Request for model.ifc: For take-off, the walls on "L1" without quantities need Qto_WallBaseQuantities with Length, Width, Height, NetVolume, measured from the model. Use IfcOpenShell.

First a look at what the model holds.

```python
import ifcopenshell
import ifcopenshell.util.element
import ifcopenshell.util.unit

model = ifcopenshell.open("model.ifc")
print(model.schema)
for unit_type in ("LENGTHUNIT", "AREAUNIT", "VOLUMEUNIT"):
    print(unit_type, ifcopenshell.util.unit.calculate_unit_scale(model, unit_type))
storey = next(s for s in model.by_type("IfcBuildingStorey") if s.Name == "L1")
walls = [e for e in ifcopenshell.util.element.get_decomposition(storey) if e.is_a("IfcWall")]
for e in sorted(walls, key=lambda e: e.id()):
    print(e.id(), e.is_a(), e.Name, list(ifcopenshell.util.element.get_psets(e, qtos_only=True)), sep=" | ")
```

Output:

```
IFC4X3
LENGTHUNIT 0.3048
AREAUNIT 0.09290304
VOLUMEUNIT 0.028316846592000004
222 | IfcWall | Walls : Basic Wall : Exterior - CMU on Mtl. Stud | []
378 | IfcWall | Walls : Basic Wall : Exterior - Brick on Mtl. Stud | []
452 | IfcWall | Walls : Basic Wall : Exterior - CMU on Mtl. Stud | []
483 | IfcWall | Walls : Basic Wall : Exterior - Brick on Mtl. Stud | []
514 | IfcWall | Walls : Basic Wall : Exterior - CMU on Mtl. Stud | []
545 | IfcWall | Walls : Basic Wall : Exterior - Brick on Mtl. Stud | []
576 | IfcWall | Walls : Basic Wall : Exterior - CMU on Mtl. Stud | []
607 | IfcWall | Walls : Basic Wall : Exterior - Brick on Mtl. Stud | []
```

```python
import ifcopenshell
import ifcopenshell.api.pset
import ifcopenshell.geom
import ifcopenshell.util.element
import ifcopenshell.util.shape
import ifcopenshell.util.unit

model = ifcopenshell.open("model.ifc")
unit_scale = ifcopenshell.util.unit.calculate_unit_scale(model)
volume_scale = ifcopenshell.util.unit.calculate_unit_scale(model, "VOLUMEUNIT")
settings = ifcopenshell.geom.settings()

storey = next(s for s in model.by_type("IfcBuildingStorey") if s.Name == "L1")
walls = [e for e in ifcopenshell.util.element.get_decomposition(storey) if e.is_a("IfcWall")]

for e in sorted(walls, key=lambda e: e.id()):
    if ifcopenshell.util.element.get_psets(e, qtos_only=True, should_inherit=False):
        continue
    # Geometry comes back in metres, in the element's own axes.
    shape = ifcopenshell.geom.create_shape(settings, e)
    values = {
        "Length": ifcopenshell.util.shape.get_x(shape.geometry) / unit_scale,
        "Width": ifcopenshell.util.shape.get_y(shape.geometry) / unit_scale,
        "Height": ifcopenshell.util.shape.get_z(shape.geometry) / unit_scale,
        "NetVolume": ifcopenshell.util.shape.get_volume(shape.geometry) / volume_scale,
    }
    qto = ifcopenshell.api.pset.add_qto(model, product=e, name="Qto_WallBaseQuantities")
    ifcopenshell.api.pset.edit_qto(model, qto=qto, properties=values)
    print(e.id(), {k: round(v, 3) for k, v in values.items()})

model.write("model_rev.ifc")
```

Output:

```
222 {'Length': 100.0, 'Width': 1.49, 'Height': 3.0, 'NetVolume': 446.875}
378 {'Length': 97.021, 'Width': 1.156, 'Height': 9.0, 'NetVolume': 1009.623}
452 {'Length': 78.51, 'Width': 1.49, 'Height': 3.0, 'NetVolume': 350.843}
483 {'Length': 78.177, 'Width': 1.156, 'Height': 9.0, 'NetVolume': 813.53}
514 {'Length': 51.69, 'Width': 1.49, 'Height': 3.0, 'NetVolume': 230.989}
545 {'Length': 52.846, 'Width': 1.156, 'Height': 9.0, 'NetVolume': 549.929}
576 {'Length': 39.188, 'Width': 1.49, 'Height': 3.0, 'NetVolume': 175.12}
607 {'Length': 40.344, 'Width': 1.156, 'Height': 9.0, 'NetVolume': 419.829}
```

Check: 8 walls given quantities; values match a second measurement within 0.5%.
